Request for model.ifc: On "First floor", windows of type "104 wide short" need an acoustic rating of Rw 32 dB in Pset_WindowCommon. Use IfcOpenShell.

First a look at what the model holds.

```python
import ifcopenshell
import ifcopenshell.util.element

model = ifcopenshell.open("model.ifc")
print(model.schema)
storey = next(s for s in model.by_type("IfcBuildingStorey") if s.Name == "First floor")
windows = [e for e in ifcopenshell.util.element.get_decomposition(storey) if e.is_a("IfcWindow")]
seen = {}
for e in windows:
    element_type = ifcopenshell.util.element.get_type(e)
    key = (element_type.Name if element_type != e and element_type else None, ifcopenshell.util.element.get_pset(e, "Pset_WindowCommon", "AcousticRating"))
    seen[key] = seen.get(key, 0) + 1
for (name, value), count in sorted(seen.items(), key=str):
    print(count, "x", name, "|", value)
```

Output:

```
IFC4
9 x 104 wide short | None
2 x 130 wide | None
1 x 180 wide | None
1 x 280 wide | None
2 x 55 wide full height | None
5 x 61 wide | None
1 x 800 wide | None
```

```python
import ifcopenshell
import ifcopenshell.api.pset
import ifcopenshell.util.element

model = ifcopenshell.open("model.ifc")

storey = next(s for s in model.by_type("IfcBuildingStorey") if s.Name == "First floor")
windows = [e for e in ifcopenshell.util.element.get_decomposition(storey) if e.is_a("IfcWindow")]

count = 0
for e in windows:
    element_type = ifcopenshell.util.element.get_type(e)
    if element_type in (None, e) or element_type.Name != "104 wide short":
        continue
    # add_pset returns the element's existing set when there is one.
    pset = ifcopenshell.api.pset.add_pset(model, product=e, name="Pset_WindowCommon")
    ifcopenshell.api.pset.edit_pset(model, pset=pset, properties={"AcousticRating": "Rw 32 dB"})
    count += 1

print(count, "windows updated")

model.write("model_updated.ifc")
```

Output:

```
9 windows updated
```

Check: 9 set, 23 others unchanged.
